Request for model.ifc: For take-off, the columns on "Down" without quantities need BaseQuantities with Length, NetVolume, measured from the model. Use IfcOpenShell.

First a look at what the model holds.

```python
import ifcopenshell
import ifcopenshell.util.element
import ifcopenshell.util.unit

model = ifcopenshell.open("model.ifc")
print(model.schema)
for unit_type in ("LENGTHUNIT", "AREAUNIT", "VOLUMEUNIT"):
    print(unit_type, ifcopenshell.util.unit.calculate_unit_scale(model, unit_type))
storey = next(s for s in model.by_type("IfcBuildingStorey") if s.Name == "Down")
columns = [e for e in ifcopenshell.util.element.get_decomposition(storey) if e.is_a("IfcColumn")]
for e in sorted(columns, key=lambda e: e.id()):
    print(e.id(), e.is_a(), e.Name, list(ifcopenshell.util.element.get_psets(e, qtos_only=True)), sep=" | ")
```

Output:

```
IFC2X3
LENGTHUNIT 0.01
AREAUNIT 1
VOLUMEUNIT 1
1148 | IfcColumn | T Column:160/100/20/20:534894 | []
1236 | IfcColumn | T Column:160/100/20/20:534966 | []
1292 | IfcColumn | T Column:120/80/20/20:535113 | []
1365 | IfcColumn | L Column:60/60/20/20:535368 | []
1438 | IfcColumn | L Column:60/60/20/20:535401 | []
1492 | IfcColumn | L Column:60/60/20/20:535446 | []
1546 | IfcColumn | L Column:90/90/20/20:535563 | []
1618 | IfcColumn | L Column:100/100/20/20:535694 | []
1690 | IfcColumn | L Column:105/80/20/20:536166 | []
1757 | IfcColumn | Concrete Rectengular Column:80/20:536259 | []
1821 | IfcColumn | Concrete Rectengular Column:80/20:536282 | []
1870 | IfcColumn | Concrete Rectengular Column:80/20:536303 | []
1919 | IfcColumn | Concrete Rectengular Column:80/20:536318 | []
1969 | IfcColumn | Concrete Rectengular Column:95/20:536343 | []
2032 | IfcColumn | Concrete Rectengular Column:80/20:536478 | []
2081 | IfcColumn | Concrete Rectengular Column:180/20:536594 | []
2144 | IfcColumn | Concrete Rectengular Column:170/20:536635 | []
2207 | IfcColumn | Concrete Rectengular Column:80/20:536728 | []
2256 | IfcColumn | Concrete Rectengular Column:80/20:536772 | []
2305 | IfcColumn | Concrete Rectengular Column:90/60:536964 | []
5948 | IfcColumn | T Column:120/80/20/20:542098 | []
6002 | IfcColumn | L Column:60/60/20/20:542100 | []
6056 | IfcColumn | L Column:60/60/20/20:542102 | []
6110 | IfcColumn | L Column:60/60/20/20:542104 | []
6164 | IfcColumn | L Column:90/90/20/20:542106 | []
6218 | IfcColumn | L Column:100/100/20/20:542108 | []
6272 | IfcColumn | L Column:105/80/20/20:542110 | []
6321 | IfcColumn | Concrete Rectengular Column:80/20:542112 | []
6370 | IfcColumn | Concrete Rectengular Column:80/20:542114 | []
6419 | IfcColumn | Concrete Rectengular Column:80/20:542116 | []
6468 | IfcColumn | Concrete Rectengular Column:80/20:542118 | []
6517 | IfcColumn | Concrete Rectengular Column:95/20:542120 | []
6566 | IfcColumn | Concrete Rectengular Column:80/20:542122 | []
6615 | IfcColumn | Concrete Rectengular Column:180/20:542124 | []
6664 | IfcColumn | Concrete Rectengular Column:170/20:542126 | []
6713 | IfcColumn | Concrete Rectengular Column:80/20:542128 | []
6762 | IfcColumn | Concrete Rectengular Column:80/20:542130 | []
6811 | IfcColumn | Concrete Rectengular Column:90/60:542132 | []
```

```python
import ifcopenshell
import ifcopenshell.api.pset
import ifcopenshell.geom
import ifcopenshell.util.element
import ifcopenshell.util.shape
import ifcopenshell.util.unit

model = ifcopenshell.open("model.ifc")
unit_scale = ifcopenshell.util.unit.calculate_unit_scale(model)
volume_scale = ifcopenshell.util.unit.calculate_unit_scale(model, "VOLUMEUNIT")
settings = ifcopenshell.geom.settings()

storey = next(s for s in model.by_type("IfcBuildingStorey") if s.Name == "Down")
columns = [e for e in ifcopenshell.util.element.get_decomposition(storey) if e.is_a("IfcColumn")]

for e in sorted(columns, key=lambda e: e.id()):
    if ifcopenshell.util.element.get_psets(e, qtos_only=True, should_inherit=False):
        continue
    # Geometry comes back in metres, in the element's own axes.
    shape = ifcopenshell.geom.create_shape(settings, e)
    values = {
        "Length": ifcopenshell.util.shape.get_z(shape.geometry) / unit_scale,
        "NetVolume": ifcopenshell.util.shape.get_volume(shape.geometry) / volume_scale,
    }
    qto = ifcopenshell.api.pset.add_qto(model, product=e, name="BaseQuantities")
    ifcopenshell.api.pset.edit_qto(model, qto=qto, properties=values)
    print(e.id(), {k: round(v, 3) for k, v in values.items()})

model.write("model_edited.ifc")
```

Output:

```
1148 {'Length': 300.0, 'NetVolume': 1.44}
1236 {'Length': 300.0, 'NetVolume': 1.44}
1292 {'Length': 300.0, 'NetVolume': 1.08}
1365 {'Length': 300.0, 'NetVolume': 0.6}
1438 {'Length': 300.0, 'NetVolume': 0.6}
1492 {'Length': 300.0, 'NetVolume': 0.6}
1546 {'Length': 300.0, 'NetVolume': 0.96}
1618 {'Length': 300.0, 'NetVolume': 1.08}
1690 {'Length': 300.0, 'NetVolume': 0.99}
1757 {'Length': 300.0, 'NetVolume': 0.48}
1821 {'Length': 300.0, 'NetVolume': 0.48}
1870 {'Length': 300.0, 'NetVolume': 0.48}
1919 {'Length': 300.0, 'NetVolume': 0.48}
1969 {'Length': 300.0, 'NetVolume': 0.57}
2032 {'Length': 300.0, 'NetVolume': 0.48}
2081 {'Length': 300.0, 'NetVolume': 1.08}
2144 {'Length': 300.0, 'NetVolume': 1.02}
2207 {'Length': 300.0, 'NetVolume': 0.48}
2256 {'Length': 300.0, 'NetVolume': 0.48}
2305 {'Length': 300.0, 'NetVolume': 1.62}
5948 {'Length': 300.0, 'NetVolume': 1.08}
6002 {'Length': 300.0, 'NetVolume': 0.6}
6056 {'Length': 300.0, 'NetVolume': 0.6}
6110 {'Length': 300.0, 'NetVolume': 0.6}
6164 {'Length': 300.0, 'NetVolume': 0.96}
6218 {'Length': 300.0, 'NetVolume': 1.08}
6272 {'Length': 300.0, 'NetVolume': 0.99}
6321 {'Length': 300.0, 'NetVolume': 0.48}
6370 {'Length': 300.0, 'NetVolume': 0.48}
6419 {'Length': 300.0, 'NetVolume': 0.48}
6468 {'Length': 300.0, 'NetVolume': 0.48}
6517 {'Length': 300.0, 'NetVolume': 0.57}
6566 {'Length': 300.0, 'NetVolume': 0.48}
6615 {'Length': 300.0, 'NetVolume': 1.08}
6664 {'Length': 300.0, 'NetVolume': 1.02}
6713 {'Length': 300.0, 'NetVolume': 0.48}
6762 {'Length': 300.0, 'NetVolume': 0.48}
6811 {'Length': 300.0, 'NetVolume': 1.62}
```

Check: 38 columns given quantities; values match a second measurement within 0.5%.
